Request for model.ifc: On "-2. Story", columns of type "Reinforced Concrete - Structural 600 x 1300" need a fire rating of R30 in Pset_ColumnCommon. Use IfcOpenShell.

First a look at what the model holds.

```python
import ifcopenshell
import ifcopenshell.util.element

model = ifcopenshell.open("model.ifc")
print(model.schema)
storey = next(s for s in model.by_type("IfcBuildingStorey") if s.Name == "-2. Story")
columns = [e for e in ifcopenshell.util.element.get_decomposition(storey) if e.is_a("IfcColumn")]
seen = {}
for e in columns:
    element_type = ifcopenshell.util.element.get_type(e)
    key = (element_type.Name if element_type != e and element_type else None, ifcopenshell.util.element.get_pset(e, "Pset_ColumnCommon", "FireRating"))
    seen[key] = seen.get(key, 0) + 1
for (name, value), count in sorted(seen.items(), key=str):
    print(count, "x", name, "|", value)
```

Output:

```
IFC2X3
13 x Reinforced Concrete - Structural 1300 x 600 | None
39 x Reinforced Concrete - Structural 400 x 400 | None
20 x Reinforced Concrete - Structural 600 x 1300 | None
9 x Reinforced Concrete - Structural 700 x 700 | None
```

```python
import ifcopenshell
import ifcopenshell.api.pset
import ifcopenshell.util.element

model = ifcopenshell.open("model.ifc")

storey = next(s for s in model.by_type("IfcBuildingStorey") if s.Name == "-2. Story")
columns = [e for e in ifcopenshell.util.element.get_decomposition(storey) if e.is_a("IfcColumn")]

count = 0
for e in columns:
    element_type = ifcopenshell.util.element.get_type(e)
    if element_type in (None, e) or element_type.Name != "Reinforced Concrete - Structural 600 x 1300":
        continue
    # add_pset returns the element's existing set when there is one.
    pset = ifcopenshell.api.pset.add_pset(model, product=e, name="Pset_ColumnCommon")
    ifcopenshell.api.pset.edit_pset(model, pset=pset, properties={"FireRating": "R30"})
    count += 1

print(count, "columns updated")

model.write("model_edited.ifc")
```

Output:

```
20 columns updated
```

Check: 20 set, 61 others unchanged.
